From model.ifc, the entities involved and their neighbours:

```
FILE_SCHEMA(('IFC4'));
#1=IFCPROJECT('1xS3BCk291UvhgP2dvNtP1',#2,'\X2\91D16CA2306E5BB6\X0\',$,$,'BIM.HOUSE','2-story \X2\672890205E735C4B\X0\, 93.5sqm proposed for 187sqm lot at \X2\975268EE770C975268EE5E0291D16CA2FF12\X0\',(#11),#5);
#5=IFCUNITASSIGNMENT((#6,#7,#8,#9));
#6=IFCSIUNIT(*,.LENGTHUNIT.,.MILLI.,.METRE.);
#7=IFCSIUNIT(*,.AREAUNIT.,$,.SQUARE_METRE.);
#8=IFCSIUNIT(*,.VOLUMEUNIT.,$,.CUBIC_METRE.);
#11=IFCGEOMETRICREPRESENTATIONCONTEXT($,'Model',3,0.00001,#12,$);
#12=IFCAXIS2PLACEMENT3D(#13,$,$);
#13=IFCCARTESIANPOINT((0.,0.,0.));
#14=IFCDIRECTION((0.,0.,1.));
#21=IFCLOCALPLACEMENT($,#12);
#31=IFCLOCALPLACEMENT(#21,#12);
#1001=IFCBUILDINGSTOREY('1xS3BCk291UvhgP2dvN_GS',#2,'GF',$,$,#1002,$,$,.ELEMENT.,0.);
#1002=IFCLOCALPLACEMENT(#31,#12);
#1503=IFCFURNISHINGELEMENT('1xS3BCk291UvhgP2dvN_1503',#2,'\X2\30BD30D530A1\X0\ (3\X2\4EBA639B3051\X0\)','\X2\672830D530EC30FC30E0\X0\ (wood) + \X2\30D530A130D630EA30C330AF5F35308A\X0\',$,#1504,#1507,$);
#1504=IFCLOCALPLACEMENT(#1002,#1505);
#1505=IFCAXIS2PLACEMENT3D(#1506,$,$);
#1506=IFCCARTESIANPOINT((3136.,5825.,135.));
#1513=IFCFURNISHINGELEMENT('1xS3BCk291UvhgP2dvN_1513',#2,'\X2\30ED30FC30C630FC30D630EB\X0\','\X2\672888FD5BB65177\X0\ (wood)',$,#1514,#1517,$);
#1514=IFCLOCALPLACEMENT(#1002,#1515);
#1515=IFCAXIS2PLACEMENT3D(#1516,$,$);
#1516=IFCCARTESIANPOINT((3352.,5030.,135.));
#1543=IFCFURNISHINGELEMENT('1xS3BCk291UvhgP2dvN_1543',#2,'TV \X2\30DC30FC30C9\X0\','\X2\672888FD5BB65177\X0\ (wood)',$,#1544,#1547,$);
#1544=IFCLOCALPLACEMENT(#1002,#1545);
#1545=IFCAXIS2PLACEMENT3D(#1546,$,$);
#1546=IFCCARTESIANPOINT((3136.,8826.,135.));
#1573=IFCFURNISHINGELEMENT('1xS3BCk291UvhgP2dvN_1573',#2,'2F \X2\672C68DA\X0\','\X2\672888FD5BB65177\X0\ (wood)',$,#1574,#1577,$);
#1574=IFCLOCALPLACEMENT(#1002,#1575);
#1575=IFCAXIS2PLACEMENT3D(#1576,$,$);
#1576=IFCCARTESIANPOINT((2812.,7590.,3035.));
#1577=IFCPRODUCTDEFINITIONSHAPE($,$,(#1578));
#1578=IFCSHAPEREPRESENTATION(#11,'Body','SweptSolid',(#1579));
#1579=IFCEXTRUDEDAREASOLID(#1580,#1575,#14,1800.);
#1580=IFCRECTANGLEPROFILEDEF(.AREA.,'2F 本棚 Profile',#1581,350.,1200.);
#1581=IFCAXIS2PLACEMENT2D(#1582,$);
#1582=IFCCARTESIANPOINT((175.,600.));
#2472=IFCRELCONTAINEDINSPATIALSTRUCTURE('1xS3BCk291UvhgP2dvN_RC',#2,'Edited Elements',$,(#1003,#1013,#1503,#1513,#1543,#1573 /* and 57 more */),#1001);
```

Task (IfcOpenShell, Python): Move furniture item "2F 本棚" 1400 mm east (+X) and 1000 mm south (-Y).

```python
import ifcopenshell
import ifcopenshell.api.geometry
import ifcopenshell.util.placement
import ifcopenshell.util.unit

model = ifcopenshell.open("model.ifc")
unit_scale = ifcopenshell.util.unit.calculate_unit_scale(model)

item = model.by_guid("1xS3BCk291UvhgP2dvN_1573")
matrix = ifcopenshell.util.placement.get_local_placement(item.ObjectPlacement)
matrix[0, 3] += 1.4 / unit_scale
matrix[1, 3] -= 1 / unit_scale
ifcopenshell.api.geometry.edit_object_placement(model, product=item, matrix=matrix, is_si=False)

print(ifcopenshell.util.placement.get_local_placement(item.ObjectPlacement).round(3) + 0.0)

model.write("model_edited.ifc")
```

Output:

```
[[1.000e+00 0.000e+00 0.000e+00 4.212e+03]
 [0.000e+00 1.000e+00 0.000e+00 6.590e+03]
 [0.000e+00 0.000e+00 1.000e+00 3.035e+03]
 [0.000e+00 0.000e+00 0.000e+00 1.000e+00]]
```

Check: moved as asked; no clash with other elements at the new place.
